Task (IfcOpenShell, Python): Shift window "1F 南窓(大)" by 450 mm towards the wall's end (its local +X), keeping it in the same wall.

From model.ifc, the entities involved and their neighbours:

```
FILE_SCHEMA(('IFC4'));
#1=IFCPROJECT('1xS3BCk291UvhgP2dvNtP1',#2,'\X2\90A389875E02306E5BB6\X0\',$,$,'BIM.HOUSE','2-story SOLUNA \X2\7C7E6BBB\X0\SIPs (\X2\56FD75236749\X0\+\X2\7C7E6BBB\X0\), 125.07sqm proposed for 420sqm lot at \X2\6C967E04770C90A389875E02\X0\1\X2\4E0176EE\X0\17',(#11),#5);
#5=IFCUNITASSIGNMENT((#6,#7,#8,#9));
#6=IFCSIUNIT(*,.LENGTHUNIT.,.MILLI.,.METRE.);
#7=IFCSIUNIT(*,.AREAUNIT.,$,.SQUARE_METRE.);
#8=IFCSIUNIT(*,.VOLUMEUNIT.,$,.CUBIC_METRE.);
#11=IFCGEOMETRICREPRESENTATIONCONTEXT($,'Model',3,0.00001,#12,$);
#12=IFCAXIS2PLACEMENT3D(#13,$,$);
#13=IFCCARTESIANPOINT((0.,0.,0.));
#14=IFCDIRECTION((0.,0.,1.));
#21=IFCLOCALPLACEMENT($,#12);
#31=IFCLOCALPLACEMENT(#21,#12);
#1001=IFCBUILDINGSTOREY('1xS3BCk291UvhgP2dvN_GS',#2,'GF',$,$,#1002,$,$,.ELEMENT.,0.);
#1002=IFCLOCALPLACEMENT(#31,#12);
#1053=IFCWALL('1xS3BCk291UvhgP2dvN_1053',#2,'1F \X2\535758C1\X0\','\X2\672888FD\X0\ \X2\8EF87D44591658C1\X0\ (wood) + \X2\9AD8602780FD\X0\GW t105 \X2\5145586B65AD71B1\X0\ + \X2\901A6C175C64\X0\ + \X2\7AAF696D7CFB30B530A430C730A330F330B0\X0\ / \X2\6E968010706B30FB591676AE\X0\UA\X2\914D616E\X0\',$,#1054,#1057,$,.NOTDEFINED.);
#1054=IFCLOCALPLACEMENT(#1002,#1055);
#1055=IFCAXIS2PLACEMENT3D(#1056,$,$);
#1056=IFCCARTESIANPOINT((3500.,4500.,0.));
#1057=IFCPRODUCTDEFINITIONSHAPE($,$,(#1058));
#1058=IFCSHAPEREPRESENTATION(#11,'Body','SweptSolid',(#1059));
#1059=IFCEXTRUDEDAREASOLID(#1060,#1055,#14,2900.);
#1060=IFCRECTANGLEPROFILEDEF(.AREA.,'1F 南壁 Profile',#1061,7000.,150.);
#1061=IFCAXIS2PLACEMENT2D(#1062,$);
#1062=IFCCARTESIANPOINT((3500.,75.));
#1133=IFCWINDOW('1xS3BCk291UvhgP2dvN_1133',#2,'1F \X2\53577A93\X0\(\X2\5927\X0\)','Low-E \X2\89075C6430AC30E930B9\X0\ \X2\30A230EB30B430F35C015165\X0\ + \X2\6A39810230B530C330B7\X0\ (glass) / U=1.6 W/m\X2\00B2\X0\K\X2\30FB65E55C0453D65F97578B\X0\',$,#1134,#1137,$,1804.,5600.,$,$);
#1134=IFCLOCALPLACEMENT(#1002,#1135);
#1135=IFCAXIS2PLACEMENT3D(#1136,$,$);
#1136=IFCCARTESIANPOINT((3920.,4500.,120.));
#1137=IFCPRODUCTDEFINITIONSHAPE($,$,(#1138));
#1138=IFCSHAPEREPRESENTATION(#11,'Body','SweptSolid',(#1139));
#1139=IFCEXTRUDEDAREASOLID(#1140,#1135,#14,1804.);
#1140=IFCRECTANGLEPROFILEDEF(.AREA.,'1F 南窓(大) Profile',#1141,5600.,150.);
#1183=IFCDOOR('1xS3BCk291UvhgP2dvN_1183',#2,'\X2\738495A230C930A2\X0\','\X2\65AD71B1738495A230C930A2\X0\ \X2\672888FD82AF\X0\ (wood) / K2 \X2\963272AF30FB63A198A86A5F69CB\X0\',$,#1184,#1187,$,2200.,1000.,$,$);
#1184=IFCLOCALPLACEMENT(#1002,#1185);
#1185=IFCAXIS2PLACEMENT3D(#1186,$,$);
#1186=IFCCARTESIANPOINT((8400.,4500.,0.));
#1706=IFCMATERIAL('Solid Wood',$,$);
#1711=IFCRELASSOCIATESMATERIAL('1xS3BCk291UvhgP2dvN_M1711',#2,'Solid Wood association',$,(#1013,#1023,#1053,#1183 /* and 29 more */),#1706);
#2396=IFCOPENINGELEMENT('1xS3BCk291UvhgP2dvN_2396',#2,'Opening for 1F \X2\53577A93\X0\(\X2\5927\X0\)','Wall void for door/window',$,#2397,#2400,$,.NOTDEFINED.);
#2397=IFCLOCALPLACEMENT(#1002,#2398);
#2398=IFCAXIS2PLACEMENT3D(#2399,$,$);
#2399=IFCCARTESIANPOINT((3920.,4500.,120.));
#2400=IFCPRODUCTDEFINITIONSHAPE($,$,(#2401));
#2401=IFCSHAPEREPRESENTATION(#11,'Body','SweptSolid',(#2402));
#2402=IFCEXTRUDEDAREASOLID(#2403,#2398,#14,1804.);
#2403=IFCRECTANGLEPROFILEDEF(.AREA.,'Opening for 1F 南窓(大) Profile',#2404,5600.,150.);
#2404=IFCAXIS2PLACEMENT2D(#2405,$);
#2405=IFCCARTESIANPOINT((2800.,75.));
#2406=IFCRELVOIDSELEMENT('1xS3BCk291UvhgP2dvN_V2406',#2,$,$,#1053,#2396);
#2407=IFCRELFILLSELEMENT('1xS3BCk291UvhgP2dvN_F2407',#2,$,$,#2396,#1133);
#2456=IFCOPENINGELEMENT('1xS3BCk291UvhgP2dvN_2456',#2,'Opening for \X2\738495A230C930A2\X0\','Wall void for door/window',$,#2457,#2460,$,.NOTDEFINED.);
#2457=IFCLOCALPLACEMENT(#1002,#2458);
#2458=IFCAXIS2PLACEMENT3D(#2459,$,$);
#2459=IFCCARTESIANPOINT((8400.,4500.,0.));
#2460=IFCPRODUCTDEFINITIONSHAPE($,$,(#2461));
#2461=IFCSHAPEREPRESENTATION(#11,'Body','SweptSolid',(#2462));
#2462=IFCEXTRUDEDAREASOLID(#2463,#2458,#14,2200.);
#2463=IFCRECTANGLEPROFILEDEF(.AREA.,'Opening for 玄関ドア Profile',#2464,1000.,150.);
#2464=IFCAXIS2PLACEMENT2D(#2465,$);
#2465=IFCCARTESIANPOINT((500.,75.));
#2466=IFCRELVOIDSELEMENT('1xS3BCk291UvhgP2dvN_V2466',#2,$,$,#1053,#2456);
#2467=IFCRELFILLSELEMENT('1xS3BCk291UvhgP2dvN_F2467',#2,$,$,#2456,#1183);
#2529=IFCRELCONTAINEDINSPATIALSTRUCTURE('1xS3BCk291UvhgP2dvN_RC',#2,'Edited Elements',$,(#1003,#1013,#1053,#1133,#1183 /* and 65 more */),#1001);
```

```python
import ifcopenshell
import ifcopenshell.api.geometry
import ifcopenshell.util.placement
import ifcopenshell.util.unit

model = ifcopenshell.open("model.ifc")
unit_scale = ifcopenshell.util.unit.calculate_unit_scale(model)

window = model.by_guid("1xS3BCk291UvhgP2dvN_1133")
opening = window.FillsVoids[0].RelatingOpeningElement
wall = opening.VoidsElements[0].RelatingBuildingElement

wall_matrix = ifcopenshell.util.placement.get_local_placement(wall.ObjectPlacement)
shift = wall_matrix[:3, 0] * 0.45 / unit_scale
before = ifcopenshell.util.placement.get_local_placement(window.ObjectPlacement)[:3, 3].copy()

# The window is not placed relative to its opening, so move both.
for product in (opening, window):
    matrix = ifcopenshell.util.placement.get_local_placement(product.ObjectPlacement)
    matrix[:3, 3] += shift
    ifcopenshell.api.geometry.edit_object_placement(model, product=product, matrix=matrix, is_si=False)

after = ifcopenshell.util.placement.get_local_placement(window.ObjectPlacement)[:3, 3]
print("window moved by", (after - before).round(3) + 0.0)

model.write("model_v2.ifc")
```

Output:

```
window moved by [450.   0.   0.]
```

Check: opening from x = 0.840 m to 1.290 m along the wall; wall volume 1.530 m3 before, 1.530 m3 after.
